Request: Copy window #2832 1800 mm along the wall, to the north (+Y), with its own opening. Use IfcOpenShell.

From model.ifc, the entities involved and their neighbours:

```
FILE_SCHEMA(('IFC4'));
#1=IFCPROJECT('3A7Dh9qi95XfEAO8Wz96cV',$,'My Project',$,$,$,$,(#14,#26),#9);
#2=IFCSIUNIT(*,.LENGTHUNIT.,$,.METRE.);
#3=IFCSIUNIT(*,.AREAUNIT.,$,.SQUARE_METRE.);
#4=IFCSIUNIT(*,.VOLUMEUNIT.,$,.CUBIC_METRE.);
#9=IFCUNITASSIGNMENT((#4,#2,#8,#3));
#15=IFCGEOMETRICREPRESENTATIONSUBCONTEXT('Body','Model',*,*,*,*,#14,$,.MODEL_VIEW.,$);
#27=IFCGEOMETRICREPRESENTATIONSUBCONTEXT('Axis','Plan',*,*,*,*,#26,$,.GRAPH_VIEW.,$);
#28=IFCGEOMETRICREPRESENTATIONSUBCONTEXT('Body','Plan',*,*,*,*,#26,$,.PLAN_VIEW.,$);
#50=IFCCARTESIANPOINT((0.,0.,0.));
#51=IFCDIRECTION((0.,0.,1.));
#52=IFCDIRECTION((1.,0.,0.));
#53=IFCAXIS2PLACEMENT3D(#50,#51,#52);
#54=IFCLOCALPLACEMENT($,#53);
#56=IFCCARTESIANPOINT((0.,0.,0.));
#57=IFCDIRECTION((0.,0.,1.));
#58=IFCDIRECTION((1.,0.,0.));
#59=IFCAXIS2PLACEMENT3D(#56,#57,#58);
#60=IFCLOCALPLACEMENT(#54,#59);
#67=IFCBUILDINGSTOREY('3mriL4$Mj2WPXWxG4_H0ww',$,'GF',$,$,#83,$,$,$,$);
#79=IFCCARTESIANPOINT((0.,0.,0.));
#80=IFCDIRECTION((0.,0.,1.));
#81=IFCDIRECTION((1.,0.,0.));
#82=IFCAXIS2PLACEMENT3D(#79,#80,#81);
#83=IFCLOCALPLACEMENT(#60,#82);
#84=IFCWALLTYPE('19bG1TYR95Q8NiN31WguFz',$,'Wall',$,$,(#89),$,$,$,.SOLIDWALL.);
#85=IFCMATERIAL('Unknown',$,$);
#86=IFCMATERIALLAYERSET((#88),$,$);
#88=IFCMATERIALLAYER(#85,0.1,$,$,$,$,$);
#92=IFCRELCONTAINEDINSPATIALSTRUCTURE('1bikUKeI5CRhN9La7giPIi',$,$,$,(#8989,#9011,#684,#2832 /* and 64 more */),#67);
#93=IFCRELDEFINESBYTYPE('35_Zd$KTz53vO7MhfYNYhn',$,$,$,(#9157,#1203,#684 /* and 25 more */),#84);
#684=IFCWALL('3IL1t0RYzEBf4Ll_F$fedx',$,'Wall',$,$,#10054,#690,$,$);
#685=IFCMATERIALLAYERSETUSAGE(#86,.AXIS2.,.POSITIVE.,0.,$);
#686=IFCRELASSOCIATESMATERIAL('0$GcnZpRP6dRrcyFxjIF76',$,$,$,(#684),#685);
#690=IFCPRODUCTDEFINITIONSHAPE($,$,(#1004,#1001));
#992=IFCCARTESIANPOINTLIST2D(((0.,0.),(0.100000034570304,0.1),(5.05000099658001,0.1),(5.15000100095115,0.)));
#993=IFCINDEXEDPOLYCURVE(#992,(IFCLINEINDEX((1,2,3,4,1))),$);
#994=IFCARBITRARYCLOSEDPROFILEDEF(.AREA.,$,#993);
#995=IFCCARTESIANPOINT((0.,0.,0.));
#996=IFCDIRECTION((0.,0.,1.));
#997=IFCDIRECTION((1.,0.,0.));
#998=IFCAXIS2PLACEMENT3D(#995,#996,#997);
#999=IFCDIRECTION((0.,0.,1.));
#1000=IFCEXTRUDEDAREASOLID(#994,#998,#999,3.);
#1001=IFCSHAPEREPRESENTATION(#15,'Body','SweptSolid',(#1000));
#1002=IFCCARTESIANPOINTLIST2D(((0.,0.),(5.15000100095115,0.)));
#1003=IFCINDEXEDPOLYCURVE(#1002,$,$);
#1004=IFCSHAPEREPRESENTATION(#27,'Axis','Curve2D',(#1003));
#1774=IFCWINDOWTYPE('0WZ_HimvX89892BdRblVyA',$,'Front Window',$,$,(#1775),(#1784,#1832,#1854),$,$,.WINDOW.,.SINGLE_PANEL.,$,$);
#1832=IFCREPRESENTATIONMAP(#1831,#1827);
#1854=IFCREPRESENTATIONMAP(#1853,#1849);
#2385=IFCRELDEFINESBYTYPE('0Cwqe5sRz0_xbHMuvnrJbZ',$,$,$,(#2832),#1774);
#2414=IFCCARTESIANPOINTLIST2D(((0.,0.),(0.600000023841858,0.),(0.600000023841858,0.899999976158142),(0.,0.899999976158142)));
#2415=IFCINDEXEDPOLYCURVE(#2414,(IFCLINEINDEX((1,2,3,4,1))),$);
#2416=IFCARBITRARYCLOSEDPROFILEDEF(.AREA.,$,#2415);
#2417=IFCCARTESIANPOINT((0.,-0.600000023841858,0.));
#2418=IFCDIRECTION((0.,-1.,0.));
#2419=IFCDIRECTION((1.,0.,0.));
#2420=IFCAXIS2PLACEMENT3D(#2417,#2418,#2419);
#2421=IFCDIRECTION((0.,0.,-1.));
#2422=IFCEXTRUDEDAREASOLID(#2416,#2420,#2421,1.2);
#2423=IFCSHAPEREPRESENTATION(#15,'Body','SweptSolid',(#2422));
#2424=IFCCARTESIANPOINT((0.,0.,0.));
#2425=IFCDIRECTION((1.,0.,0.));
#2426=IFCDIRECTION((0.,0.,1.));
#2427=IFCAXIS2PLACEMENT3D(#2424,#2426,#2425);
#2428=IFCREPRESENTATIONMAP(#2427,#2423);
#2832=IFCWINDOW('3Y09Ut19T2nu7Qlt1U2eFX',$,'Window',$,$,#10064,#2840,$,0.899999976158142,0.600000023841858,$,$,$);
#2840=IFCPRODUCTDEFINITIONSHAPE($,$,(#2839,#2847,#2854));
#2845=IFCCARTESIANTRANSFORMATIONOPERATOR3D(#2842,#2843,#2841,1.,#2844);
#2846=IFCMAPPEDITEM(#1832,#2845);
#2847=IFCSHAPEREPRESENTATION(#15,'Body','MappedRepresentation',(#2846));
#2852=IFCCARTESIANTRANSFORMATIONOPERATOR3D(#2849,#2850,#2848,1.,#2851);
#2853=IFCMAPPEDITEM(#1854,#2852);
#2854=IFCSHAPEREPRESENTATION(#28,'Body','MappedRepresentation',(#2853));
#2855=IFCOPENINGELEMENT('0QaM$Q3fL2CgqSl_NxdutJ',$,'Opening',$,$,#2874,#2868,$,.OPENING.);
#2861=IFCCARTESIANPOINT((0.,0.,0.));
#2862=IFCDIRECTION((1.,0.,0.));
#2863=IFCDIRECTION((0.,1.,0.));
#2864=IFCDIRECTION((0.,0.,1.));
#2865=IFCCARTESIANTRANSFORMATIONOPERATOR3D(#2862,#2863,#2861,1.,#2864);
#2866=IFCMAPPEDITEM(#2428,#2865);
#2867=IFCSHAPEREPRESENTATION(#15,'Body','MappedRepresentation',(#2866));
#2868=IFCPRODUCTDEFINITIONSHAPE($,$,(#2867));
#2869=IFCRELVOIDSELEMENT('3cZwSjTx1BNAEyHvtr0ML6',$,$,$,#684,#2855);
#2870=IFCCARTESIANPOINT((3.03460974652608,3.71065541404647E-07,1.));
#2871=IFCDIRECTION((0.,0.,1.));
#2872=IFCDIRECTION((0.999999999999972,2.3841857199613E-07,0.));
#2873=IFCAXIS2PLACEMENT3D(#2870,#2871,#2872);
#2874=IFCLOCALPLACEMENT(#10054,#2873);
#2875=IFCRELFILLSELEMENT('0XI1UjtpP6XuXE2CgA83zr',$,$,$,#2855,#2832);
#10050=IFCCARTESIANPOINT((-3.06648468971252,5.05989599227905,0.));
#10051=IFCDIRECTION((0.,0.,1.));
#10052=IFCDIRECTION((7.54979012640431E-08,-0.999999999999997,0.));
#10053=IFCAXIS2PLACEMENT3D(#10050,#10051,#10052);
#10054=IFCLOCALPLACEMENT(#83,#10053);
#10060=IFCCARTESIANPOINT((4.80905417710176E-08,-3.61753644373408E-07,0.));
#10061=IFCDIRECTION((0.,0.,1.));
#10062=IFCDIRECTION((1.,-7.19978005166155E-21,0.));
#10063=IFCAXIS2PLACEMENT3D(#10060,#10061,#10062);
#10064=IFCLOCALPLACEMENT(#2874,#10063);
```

```python
import ifcopenshell
import ifcopenshell.api.feature
import ifcopenshell.api.geometry
import ifcopenshell.api.root
import ifcopenshell.geom
import ifcopenshell.util.element
import ifcopenshell.util.placement
import ifcopenshell.util.shape
import ifcopenshell.util.unit

model = ifcopenshell.open("model.ifc")
unit_scale = ifcopenshell.util.unit.calculate_unit_scale(model)
settings = ifcopenshell.geom.settings()


def volume(element):
    """Net volume in cubic metres, openings subtracted."""
    shape = ifcopenshell.geom.create_shape(settings, element)
    return ifcopenshell.util.shape.get_volume(shape.geometry)


window = model.by_guid("3Y09Ut19T2nu7Qlt1U2eFX")
opening = window.FillsVoids[0].RelatingOpeningElement
wall = opening.VoidsElements[0].RelatingBuildingElement
before = volume(wall)
shift = ifcopenshell.util.placement.get_local_placement(wall.ObjectPlacement)[:3, 0] * -1.8 / unit_scale

# copy_class copies the void relationship, type, container and properties, but no geometry.
new_opening = ifcopenshell.api.root.copy_class(model, product=opening)
new_opening.Representation = ifcopenshell.util.element.copy_deep(
    model, opening.Representation, exclude=["IfcGeometricRepresentationContext", "IfcRepresentationMap"]
)
new_window = ifcopenshell.api.root.copy_class(model, product=window)
new_window.Representation = ifcopenshell.util.element.copy_deep(
    model, window.Representation, exclude=["IfcGeometricRepresentationContext", "IfcRepresentationMap"]
)
ifcopenshell.api.feature.add_filling(model, opening=new_opening, element=new_window)

for old, new in ((opening, new_opening), (window, new_window)):
    matrix = ifcopenshell.util.placement.get_local_placement(old.ObjectPlacement)
    matrix[:3, 3] += shift
    ifcopenshell.api.geometry.edit_object_placement(model, product=new, matrix=matrix, is_si=False)

after = volume(wall)

print(f"wall volume {before:.3f} -> {after:.3f} m3")

model.write("model_rev.ifc")
```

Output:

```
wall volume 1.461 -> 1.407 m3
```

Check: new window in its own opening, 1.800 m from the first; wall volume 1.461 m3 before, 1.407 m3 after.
